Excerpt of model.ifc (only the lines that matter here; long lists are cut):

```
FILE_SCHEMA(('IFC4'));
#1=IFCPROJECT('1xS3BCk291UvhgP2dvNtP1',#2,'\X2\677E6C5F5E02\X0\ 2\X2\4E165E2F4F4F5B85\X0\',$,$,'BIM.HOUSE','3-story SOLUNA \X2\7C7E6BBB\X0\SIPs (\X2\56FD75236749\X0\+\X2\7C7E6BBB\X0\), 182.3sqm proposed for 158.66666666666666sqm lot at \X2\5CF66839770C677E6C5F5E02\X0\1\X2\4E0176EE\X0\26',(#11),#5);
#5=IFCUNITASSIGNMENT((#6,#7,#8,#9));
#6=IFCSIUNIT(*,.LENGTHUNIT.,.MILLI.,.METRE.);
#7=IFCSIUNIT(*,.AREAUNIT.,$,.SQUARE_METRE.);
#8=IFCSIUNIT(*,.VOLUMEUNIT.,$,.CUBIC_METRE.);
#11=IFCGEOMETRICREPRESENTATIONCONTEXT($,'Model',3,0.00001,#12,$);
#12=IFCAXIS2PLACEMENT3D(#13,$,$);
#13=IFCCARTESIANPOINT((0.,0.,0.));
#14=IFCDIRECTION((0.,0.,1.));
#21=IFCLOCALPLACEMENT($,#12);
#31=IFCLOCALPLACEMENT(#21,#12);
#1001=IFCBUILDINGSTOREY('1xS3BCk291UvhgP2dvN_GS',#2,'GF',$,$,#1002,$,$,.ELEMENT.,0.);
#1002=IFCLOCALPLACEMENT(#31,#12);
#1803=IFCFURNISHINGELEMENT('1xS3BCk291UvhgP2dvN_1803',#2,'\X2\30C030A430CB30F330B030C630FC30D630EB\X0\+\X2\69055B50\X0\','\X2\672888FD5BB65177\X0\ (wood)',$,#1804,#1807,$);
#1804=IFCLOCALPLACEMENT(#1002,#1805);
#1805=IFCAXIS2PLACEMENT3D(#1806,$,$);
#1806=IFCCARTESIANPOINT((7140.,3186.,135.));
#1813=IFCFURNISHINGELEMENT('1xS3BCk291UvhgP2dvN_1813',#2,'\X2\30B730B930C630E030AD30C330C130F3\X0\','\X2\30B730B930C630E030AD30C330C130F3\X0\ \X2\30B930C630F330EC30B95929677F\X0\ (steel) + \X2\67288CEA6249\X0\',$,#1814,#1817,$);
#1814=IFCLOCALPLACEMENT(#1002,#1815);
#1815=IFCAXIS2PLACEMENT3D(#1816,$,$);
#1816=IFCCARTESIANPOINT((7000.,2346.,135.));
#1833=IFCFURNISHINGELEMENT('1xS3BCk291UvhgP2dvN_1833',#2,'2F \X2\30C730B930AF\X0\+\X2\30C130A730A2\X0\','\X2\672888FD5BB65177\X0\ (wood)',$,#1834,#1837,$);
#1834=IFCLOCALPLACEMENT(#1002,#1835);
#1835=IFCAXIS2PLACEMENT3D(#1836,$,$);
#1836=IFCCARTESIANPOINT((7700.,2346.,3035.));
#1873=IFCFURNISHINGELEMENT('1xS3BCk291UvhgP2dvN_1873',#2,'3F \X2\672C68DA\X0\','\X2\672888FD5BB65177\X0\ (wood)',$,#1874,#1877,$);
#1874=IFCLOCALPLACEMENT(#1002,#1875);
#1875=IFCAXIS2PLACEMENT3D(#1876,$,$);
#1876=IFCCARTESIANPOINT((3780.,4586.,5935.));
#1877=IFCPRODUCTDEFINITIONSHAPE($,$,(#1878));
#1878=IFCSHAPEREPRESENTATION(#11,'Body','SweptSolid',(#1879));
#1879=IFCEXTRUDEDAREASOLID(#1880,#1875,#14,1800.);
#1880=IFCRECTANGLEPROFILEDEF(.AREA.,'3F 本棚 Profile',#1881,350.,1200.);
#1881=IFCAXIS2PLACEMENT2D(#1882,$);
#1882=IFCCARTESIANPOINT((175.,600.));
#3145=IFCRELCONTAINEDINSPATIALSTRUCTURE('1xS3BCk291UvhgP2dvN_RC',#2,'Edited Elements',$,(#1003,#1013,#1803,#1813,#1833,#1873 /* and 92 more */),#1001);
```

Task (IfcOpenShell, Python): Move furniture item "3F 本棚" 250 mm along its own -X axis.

```python
import ifcopenshell
import ifcopenshell.api.geometry
import ifcopenshell.util.placement
import ifcopenshell.util.unit

model = ifcopenshell.open("model.ifc")
unit_scale = ifcopenshell.util.unit.calculate_unit_scale(model)

item = model.by_guid("1xS3BCk291UvhgP2dvN_1873")
matrix = ifcopenshell.util.placement.get_local_placement(item.ObjectPlacement)
matrix[:3, 3] -= matrix[:3, 0] * 0.25 / unit_scale
ifcopenshell.api.geometry.edit_object_placement(model, product=item, matrix=matrix, is_si=False)

print(ifcopenshell.util.placement.get_local_placement(item.ObjectPlacement).round(3) + 0.0)

model.write("model_rev.ifc")
```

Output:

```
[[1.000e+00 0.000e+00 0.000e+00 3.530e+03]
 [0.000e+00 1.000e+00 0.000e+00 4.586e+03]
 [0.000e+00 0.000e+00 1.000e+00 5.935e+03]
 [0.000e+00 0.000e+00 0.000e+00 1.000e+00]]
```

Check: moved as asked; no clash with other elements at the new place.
